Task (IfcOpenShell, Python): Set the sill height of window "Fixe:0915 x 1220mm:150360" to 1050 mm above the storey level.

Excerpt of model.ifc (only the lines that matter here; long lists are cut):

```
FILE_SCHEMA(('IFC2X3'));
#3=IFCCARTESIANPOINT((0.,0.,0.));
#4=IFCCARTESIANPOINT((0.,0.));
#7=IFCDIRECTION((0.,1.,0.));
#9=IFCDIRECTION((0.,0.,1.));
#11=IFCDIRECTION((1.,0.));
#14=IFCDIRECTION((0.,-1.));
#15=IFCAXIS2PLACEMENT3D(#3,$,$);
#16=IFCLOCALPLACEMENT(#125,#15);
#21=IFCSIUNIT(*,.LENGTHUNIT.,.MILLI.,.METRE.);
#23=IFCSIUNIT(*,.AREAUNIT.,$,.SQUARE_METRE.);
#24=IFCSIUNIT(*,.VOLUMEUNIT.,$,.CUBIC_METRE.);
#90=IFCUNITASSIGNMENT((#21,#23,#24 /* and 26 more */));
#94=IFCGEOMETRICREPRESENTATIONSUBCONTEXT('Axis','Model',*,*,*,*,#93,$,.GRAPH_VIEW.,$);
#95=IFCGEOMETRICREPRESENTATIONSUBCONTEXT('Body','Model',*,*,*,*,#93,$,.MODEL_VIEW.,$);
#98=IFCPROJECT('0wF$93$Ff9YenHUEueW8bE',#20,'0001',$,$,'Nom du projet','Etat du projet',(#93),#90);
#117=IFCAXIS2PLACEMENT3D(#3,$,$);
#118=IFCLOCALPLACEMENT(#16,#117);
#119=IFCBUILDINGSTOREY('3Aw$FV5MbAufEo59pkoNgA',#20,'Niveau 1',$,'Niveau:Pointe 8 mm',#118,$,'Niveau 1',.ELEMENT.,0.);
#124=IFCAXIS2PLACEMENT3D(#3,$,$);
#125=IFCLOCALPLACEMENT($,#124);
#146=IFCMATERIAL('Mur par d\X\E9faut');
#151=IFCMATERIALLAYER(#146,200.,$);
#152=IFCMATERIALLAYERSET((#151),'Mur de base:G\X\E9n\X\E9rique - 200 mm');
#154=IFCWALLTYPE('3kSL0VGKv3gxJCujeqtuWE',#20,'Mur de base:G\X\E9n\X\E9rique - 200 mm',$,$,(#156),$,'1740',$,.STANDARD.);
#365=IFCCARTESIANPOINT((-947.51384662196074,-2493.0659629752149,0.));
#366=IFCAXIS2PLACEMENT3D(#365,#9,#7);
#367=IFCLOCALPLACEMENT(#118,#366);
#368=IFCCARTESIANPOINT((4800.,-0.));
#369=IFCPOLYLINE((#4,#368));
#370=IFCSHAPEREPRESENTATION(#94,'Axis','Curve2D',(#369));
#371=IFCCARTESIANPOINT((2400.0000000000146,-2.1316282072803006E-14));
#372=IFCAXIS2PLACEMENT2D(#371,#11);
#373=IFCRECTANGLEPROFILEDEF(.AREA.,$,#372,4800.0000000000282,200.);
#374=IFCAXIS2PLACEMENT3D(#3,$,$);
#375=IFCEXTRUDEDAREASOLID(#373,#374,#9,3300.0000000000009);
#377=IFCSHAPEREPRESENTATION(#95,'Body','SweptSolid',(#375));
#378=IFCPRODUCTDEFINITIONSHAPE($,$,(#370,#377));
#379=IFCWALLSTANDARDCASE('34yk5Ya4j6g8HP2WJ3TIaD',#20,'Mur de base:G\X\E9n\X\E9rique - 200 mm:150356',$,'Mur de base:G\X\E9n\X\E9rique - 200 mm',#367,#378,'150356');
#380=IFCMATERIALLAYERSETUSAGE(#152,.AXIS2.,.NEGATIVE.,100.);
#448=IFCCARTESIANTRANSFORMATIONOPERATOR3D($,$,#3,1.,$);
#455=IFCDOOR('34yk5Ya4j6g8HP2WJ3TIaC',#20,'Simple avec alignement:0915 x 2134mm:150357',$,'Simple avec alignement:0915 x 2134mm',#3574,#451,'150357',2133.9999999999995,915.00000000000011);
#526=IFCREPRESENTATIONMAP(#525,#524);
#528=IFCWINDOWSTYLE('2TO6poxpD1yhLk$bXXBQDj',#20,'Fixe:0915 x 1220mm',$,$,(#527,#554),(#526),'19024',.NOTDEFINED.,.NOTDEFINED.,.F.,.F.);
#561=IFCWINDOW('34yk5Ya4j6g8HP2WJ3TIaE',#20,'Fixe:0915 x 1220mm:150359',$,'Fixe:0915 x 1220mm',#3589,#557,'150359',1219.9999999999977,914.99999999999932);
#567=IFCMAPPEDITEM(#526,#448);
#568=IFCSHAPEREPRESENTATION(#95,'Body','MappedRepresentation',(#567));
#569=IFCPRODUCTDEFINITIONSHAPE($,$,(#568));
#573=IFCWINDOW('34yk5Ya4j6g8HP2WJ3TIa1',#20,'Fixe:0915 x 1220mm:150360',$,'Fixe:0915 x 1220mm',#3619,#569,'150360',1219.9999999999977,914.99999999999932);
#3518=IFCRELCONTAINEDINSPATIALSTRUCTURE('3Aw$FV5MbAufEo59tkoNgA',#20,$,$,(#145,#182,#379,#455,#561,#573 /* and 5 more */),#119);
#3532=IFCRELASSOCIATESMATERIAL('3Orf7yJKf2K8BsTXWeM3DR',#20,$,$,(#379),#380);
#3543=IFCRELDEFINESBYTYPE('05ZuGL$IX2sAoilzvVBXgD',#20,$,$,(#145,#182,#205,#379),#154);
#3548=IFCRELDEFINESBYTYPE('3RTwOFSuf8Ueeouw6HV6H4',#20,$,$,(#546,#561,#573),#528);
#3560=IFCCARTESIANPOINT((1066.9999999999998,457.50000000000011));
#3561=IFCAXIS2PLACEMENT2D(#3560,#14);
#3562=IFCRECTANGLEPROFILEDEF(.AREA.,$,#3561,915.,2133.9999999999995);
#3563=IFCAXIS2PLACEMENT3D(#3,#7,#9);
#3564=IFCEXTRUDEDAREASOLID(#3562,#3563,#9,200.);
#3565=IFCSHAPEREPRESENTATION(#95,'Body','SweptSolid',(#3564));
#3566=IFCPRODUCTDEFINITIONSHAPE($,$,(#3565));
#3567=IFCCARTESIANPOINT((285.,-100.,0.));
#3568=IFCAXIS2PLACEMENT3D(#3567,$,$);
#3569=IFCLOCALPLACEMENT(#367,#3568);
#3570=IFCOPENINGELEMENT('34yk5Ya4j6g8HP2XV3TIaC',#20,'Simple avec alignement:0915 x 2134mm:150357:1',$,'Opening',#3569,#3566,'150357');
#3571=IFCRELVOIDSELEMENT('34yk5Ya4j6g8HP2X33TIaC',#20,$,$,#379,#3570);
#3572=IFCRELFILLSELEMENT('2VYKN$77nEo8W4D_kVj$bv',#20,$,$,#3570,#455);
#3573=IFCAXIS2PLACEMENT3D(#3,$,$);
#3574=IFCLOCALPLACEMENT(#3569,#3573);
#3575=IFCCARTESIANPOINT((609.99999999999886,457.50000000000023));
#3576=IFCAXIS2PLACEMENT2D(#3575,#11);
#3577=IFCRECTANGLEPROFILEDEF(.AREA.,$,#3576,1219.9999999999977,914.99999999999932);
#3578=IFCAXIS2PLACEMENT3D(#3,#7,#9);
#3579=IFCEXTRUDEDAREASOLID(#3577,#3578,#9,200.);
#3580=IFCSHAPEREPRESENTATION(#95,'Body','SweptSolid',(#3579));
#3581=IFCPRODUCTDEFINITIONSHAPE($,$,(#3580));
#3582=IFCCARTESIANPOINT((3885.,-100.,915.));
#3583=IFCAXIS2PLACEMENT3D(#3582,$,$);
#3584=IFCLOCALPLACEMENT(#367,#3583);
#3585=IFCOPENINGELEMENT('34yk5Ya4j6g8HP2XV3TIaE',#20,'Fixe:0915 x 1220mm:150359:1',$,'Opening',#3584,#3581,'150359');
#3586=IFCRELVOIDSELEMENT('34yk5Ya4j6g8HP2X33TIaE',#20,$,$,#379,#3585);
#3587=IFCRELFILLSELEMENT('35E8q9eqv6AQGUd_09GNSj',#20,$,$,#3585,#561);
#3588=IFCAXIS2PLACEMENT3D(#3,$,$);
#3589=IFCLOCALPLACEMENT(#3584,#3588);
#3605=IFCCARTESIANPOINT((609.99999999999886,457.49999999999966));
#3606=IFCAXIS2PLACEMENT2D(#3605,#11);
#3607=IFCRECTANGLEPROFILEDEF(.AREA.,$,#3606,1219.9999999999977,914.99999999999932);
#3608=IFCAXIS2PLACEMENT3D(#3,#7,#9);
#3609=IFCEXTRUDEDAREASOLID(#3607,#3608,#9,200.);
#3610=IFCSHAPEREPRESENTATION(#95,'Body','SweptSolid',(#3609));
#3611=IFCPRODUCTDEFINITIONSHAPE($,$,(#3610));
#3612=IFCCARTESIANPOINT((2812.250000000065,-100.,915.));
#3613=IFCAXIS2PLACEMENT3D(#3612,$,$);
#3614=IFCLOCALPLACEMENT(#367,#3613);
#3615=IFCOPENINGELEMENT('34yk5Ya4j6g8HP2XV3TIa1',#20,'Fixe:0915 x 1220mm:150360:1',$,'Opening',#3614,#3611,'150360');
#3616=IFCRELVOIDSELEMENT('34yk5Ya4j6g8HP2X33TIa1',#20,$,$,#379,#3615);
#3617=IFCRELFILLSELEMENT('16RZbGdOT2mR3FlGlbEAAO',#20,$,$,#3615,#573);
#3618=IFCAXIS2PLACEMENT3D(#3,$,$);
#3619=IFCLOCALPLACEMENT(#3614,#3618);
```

```python
import numpy as np
import ifcopenshell
import ifcopenshell.api.geometry
import ifcopenshell.geom
import ifcopenshell.util.element
import ifcopenshell.util.placement
import ifcopenshell.util.shape
import ifcopenshell.util.unit

model = ifcopenshell.open("model.ifc")
unit_scale = ifcopenshell.util.unit.calculate_unit_scale(model)

window = model.by_guid("34yk5Ya4j6g8HP2WJ3TIa1")
opening = window.FillsVoids[0].RelatingOpeningElement
storey = ifcopenshell.util.element.get_container(window, ifc_class="IfcBuildingStorey")
level = ifcopenshell.util.placement.get_local_placement(storey.ObjectPlacement)[2, 3]

# The opening's origin need not be at the sill, so measure its lowest point.
shape = ifcopenshell.geom.create_shape(ifcopenshell.geom.settings(), opening)
bottom = ifcopenshell.util.shape.get_shape_bottom_elevation(shape, shape.geometry) / unit_scale
dz = level + 1.05 / unit_scale - bottom

shift = np.array([0.0, 0.0, dz])
# The window is placed relative to its opening, so it follows when the opening moves.
matrix = ifcopenshell.util.placement.get_local_placement(opening.ObjectPlacement)
matrix[:3, 3] += shift
ifcopenshell.api.geometry.edit_object_placement(
    model, product=opening, matrix=matrix, is_si=False, should_transform_children=True
)

print(f"moved by {dz * unit_scale:+.3f} m")

model.write("model_edited.ifc")
```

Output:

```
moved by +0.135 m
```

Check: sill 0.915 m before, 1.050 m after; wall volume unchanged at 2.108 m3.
